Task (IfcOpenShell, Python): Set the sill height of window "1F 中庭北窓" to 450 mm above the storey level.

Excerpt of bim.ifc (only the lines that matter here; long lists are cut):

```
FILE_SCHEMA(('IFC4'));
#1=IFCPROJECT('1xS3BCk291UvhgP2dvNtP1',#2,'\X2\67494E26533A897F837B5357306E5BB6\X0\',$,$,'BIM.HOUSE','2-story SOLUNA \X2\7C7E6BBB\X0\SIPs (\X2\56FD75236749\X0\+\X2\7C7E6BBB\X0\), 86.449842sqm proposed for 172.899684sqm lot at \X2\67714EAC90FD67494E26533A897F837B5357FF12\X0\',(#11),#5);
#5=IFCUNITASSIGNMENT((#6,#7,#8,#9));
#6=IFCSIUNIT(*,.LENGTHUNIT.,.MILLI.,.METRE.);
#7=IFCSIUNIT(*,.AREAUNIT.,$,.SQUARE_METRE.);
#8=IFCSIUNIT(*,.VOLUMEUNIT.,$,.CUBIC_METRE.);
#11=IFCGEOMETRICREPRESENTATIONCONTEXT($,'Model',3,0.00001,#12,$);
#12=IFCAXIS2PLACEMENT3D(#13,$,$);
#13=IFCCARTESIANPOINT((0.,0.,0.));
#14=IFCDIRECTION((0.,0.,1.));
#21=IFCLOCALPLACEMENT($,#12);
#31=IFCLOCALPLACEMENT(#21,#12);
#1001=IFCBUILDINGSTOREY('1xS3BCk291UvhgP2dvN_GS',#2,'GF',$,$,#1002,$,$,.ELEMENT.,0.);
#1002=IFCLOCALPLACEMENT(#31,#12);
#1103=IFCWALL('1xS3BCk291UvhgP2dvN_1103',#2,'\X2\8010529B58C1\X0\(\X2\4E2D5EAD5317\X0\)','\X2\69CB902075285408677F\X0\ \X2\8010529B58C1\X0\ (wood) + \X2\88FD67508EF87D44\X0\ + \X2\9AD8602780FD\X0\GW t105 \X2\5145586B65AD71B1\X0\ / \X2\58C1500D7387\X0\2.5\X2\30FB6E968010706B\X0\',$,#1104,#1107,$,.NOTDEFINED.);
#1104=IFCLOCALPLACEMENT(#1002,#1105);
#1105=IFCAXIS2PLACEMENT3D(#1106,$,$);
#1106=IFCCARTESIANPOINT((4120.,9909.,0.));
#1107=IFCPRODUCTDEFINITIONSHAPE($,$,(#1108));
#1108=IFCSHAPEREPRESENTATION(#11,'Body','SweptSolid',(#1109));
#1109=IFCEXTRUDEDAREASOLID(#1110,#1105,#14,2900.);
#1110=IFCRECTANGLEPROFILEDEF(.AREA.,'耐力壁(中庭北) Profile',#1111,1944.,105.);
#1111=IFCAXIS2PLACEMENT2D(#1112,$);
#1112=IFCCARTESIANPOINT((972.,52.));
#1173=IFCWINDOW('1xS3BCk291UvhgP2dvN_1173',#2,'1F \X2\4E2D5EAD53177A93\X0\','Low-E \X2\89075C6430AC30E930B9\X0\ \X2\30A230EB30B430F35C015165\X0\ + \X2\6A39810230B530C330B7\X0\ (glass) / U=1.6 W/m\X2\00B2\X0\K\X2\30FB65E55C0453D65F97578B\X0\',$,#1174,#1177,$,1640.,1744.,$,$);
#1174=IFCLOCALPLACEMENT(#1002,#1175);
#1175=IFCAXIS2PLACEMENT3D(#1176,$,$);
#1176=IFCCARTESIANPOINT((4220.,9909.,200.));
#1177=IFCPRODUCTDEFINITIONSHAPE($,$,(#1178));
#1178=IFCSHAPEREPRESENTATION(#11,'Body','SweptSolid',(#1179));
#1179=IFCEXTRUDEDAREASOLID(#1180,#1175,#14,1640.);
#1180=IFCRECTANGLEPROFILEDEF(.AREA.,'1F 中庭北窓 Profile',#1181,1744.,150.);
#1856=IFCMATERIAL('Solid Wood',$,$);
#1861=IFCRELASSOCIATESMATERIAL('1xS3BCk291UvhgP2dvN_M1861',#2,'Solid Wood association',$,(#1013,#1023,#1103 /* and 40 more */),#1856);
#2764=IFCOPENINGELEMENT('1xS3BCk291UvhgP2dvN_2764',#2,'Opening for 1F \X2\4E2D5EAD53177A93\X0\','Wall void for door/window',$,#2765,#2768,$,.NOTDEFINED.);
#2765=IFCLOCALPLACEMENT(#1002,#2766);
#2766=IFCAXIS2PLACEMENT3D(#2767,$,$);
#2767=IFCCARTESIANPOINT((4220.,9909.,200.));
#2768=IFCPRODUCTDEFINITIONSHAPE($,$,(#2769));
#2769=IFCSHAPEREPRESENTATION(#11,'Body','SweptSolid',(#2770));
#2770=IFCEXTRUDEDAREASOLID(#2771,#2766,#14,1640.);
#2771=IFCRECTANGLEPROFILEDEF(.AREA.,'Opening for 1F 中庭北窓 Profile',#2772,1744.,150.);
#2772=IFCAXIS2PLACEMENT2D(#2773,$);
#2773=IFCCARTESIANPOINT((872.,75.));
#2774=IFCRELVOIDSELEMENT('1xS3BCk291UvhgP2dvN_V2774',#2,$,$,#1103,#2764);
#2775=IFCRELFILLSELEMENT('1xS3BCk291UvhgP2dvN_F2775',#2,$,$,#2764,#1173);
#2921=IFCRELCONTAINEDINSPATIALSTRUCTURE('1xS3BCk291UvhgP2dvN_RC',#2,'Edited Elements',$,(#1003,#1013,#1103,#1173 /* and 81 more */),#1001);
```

```python
import numpy as np
import ifcopenshell
import ifcopenshell.api.geometry
import ifcopenshell.geom
import ifcopenshell.util.element
import ifcopenshell.util.placement
import ifcopenshell.util.shape
import ifcopenshell.util.unit

model = ifcopenshell.open("bim.ifc")
unit_scale = ifcopenshell.util.unit.calculate_unit_scale(model)

window = model.by_guid("1xS3BCk291UvhgP2dvN_1173")
opening = window.FillsVoids[0].RelatingOpeningElement
storey = ifcopenshell.util.element.get_container(window, ifc_class="IfcBuildingStorey")
level = ifcopenshell.util.placement.get_local_placement(storey.ObjectPlacement)[2, 3]

# The opening's origin need not be at the sill, so measure its lowest point.
shape = ifcopenshell.geom.create_shape(ifcopenshell.geom.settings(), opening)
bottom = ifcopenshell.util.shape.get_shape_bottom_elevation(shape, shape.geometry) / unit_scale
dz = level + 0.45 / unit_scale - bottom

shift = np.array([0.0, 0.0, dz])
# The window is not placed relative to its opening, so move both.
for product in (opening, window):
    matrix = ifcopenshell.util.placement.get_local_placement(product.ObjectPlacement)
    matrix[:3, 3] += shift
    ifcopenshell.api.geometry.edit_object_placement(model, product=product, matrix=matrix, is_si=False)

print(f"moved by {dz * unit_scale:+.3f} m")

model.write("bim-out.ifc")
```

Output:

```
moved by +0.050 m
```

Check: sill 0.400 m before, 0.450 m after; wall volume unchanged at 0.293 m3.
